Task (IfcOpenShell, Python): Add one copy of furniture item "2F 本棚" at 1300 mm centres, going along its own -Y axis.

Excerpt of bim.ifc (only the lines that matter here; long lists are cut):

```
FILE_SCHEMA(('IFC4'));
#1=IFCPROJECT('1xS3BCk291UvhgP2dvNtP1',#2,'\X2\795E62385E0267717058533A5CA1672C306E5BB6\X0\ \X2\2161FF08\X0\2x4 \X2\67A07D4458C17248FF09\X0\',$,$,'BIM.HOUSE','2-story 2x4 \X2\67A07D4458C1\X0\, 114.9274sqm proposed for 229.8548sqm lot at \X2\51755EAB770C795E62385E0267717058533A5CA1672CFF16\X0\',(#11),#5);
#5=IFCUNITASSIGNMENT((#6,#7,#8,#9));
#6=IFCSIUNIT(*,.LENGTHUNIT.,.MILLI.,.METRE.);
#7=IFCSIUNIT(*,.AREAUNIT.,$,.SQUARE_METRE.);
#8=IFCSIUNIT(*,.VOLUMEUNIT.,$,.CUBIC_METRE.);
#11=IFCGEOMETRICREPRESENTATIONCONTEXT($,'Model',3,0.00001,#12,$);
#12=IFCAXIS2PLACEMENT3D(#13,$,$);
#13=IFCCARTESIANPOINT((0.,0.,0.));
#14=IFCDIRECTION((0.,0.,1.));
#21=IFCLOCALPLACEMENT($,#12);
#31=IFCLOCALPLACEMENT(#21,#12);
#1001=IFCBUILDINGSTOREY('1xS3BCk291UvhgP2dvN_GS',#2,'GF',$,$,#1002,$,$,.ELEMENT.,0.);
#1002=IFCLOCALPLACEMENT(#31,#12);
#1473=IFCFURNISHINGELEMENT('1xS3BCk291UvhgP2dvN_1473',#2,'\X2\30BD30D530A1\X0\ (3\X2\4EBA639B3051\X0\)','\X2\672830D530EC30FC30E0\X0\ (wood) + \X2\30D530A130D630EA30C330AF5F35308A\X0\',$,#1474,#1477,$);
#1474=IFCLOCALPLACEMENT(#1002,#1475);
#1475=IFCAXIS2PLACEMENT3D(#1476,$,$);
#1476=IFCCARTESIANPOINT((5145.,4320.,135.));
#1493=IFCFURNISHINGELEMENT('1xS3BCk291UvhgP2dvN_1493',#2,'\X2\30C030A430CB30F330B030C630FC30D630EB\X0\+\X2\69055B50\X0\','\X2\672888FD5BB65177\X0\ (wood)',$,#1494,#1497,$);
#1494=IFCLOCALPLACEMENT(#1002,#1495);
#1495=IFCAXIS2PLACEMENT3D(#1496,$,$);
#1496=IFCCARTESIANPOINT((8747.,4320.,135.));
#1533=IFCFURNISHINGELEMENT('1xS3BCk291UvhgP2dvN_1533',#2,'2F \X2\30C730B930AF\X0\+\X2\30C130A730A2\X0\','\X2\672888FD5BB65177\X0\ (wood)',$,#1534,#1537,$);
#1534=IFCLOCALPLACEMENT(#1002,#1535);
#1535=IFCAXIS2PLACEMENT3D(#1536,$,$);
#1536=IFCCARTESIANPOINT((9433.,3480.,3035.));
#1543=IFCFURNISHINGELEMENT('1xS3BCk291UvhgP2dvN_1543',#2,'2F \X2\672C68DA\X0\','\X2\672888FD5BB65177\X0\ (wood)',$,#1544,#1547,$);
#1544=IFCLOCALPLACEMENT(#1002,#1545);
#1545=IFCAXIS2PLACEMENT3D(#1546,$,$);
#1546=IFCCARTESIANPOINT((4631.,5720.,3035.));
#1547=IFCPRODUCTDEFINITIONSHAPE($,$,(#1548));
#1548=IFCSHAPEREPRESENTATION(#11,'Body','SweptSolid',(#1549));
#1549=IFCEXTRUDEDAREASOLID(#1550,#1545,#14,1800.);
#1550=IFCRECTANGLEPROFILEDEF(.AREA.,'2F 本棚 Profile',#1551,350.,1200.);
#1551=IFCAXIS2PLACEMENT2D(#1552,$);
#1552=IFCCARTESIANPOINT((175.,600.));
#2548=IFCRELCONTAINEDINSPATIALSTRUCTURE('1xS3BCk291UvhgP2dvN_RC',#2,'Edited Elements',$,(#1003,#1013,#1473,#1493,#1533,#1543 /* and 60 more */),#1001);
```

```python
import ifcopenshell
import ifcopenshell.api.geometry
import ifcopenshell.api.root
import ifcopenshell.util.element
import ifcopenshell.util.placement
import ifcopenshell.util.unit

model = ifcopenshell.open("bim.ifc")
unit_scale = ifcopenshell.util.unit.calculate_unit_scale(model)


def reuse_history(source, copy):
    """copy_class also copies each property set's owner history, people and application; keep the originals."""
    for rel in copy.IsDefinedBy:
        if rel.is_a("IfcRelDefinesByProperties") and (history := rel.RelatingPropertyDefinition.OwnerHistory):
            rel.RelatingPropertyDefinition.OwnerHistory = source.OwnerHistory
            ifcopenshell.util.element.remove_deep2(model, history)


source = model.by_guid("1xS3BCk291UvhgP2dvN_1543")
base = ifcopenshell.util.placement.get_local_placement(source.ObjectPlacement)
step = -base[:3, 1] * 1.3 / unit_scale

for i in range(1, 2):
    copy = ifcopenshell.api.root.copy_class(model, product=source)
    copy.Representation = ifcopenshell.util.element.copy_deep(
        model, source.Representation, exclude=["IfcGeometricRepresentationContext", "IfcRepresentationMap"]
    )
    reuse_history(source, copy)
    matrix = base.copy()
    matrix[:3, 3] += i * step
    print("added at", matrix[:3, 3].round(3) + 0.0)
    ifcopenshell.api.geometry.edit_object_placement(model, product=copy, matrix=matrix, is_si=False)

model.write("bim-out.ifc")
```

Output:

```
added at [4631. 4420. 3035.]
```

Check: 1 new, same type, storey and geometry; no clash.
